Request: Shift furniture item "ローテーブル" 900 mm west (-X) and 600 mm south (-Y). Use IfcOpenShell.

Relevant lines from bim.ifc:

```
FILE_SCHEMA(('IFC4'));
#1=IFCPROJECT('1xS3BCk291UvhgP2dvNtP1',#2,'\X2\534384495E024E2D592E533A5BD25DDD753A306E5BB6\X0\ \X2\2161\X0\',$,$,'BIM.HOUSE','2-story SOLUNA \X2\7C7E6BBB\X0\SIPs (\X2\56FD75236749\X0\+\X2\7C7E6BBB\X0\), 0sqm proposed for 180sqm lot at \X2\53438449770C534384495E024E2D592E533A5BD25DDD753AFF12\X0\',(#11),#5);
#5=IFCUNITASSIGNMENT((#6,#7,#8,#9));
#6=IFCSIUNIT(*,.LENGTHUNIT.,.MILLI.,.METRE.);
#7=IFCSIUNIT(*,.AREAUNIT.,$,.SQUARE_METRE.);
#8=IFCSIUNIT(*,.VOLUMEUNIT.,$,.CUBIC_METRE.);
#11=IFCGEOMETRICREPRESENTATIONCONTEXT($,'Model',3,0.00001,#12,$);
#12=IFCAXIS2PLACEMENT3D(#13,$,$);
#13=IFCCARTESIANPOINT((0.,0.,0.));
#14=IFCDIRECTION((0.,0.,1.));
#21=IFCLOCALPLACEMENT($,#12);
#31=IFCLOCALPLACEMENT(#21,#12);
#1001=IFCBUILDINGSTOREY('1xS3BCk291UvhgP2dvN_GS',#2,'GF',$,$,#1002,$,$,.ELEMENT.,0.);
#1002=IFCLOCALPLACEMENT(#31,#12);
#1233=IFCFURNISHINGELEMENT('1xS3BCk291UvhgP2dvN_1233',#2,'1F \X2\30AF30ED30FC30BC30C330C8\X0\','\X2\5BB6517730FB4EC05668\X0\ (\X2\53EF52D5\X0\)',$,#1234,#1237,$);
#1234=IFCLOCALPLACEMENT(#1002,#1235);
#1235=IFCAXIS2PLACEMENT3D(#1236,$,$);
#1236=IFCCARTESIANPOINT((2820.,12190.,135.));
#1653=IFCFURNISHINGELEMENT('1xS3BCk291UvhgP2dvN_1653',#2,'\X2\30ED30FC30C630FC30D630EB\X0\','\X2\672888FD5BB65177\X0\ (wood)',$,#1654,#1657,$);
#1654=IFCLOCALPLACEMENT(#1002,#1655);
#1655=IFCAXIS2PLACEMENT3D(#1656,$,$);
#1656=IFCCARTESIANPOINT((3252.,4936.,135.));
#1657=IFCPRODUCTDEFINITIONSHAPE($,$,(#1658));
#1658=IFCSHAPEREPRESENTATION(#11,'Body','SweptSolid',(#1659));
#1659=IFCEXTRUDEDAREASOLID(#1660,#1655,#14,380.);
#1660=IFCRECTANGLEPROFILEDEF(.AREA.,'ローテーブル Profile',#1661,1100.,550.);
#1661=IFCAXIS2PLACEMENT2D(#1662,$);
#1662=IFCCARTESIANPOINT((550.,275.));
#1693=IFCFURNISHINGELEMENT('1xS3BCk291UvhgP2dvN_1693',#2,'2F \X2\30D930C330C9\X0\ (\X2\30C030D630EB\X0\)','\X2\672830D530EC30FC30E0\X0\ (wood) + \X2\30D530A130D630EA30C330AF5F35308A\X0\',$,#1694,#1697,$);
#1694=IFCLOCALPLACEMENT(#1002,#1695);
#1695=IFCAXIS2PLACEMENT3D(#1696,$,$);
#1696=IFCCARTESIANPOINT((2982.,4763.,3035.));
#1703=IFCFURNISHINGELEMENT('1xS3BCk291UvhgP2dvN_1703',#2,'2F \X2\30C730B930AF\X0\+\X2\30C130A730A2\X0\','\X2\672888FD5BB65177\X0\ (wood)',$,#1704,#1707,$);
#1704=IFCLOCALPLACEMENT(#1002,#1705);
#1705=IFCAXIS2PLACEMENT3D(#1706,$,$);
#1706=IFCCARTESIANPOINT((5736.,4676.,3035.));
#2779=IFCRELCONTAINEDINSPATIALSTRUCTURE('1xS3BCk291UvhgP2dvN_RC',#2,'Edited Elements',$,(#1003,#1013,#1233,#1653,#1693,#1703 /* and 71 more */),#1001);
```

```python
import ifcopenshell
import ifcopenshell.api.geometry
import ifcopenshell.util.placement

model = ifcopenshell.open("bim.ifc")

item = model.by_guid("1xS3BCk291UvhgP2dvN_1653")
matrix = ifcopenshell.util.placement.get_local_placement(item.ObjectPlacement)
matrix[0, 3] -= 900.0
matrix[1, 3] -= 600.0
ifcopenshell.api.geometry.edit_object_placement(model, product=item, matrix=matrix, is_si=False)

print(ifcopenshell.util.placement.get_local_placement(item.ObjectPlacement).round(3) + 0.0)

model.write("bim_v2.ifc")
```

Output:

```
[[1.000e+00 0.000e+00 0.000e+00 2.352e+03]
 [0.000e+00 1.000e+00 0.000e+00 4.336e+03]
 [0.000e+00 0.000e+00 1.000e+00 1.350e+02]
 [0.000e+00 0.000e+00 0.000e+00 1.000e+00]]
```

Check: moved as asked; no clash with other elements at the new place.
